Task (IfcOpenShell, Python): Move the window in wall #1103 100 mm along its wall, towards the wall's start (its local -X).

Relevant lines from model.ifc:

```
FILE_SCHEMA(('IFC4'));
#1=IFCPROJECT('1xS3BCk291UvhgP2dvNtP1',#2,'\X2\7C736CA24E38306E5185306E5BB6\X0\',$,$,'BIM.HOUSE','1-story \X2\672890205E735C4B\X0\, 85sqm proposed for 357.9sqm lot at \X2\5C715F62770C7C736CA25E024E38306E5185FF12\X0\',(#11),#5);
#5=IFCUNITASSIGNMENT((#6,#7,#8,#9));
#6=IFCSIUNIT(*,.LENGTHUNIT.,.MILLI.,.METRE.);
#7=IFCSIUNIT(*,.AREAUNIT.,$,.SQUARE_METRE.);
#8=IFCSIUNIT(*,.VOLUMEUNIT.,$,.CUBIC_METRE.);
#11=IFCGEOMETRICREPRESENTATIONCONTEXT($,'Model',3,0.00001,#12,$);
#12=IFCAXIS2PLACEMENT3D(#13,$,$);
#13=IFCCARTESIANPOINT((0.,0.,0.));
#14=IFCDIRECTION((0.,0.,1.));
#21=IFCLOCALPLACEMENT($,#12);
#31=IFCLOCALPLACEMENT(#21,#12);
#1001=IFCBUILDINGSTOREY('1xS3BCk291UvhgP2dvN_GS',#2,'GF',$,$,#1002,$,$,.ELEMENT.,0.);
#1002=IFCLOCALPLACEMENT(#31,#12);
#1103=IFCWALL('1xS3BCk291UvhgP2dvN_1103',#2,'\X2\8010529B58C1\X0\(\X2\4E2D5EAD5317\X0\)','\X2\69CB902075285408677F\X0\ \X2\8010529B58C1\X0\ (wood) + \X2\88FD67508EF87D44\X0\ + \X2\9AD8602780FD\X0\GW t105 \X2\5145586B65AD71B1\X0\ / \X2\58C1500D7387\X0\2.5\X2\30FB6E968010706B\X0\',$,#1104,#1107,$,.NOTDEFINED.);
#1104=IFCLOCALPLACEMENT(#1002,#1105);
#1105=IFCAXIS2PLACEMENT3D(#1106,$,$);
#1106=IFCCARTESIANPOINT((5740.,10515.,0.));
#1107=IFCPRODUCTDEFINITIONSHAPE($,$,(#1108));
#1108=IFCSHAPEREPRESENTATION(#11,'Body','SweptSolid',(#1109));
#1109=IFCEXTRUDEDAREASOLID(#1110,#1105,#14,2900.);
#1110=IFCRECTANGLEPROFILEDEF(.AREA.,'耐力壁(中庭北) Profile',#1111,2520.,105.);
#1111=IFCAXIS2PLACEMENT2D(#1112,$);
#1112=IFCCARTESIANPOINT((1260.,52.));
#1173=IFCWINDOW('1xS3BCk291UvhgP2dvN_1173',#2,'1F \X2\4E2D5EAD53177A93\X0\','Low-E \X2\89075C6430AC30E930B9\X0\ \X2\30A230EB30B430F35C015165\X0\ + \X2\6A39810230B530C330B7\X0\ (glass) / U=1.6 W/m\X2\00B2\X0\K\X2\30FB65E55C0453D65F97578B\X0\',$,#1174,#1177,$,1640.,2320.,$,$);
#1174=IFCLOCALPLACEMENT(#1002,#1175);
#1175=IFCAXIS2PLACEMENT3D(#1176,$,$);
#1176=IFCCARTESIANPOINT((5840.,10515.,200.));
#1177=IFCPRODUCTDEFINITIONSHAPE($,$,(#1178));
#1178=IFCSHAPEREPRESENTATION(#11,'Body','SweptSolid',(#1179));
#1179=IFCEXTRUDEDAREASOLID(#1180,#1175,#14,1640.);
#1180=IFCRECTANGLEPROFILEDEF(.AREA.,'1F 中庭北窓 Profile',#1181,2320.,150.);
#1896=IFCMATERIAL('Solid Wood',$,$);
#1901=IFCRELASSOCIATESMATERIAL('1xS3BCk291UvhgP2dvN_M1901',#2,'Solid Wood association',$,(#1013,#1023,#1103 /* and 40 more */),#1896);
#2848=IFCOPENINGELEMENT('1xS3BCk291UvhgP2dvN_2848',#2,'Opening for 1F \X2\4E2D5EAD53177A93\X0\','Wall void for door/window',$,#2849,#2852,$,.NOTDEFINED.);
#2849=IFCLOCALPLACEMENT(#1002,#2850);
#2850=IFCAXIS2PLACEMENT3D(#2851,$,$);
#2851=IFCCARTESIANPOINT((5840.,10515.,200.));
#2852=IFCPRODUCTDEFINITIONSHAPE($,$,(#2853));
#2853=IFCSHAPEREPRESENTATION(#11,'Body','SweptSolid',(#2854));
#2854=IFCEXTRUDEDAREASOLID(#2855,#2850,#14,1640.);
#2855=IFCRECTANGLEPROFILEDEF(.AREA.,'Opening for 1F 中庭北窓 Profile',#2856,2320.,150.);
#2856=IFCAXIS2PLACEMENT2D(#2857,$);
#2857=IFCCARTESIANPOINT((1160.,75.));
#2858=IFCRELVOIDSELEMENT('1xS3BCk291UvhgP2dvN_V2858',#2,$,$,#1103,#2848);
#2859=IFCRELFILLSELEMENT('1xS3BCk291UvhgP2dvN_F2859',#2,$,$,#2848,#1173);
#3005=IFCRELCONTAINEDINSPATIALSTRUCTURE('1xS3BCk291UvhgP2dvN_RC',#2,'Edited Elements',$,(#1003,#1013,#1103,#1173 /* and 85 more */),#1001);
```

```python
import ifcopenshell
import ifcopenshell.api.geometry
import ifcopenshell.util.placement
import ifcopenshell.util.unit

model = ifcopenshell.open("model.ifc")
unit_scale = ifcopenshell.util.unit.calculate_unit_scale(model)

window = model.by_id(1173)
opening = window.FillsVoids[0].RelatingOpeningElement
wall = opening.VoidsElements[0].RelatingBuildingElement

wall_matrix = ifcopenshell.util.placement.get_local_placement(wall.ObjectPlacement)
shift = wall_matrix[:3, 0] * -0.1 / unit_scale
before = ifcopenshell.util.placement.get_local_placement(window.ObjectPlacement)[:3, 3].copy()

# The window is not placed relative to its opening, so move both.
for product in (opening, window):
    matrix = ifcopenshell.util.placement.get_local_placement(product.ObjectPlacement)
    matrix[:3, 3] += shift
    ifcopenshell.api.geometry.edit_object_placement(model, product=product, matrix=matrix, is_si=False)

after = ifcopenshell.util.placement.get_local_placement(window.ObjectPlacement)[:3, 3]
print("window moved by", (after - before).round(3) + 0.0)

model.write("model-out.ifc")
```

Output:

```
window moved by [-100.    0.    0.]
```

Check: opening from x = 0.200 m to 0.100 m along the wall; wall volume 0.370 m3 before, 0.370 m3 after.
